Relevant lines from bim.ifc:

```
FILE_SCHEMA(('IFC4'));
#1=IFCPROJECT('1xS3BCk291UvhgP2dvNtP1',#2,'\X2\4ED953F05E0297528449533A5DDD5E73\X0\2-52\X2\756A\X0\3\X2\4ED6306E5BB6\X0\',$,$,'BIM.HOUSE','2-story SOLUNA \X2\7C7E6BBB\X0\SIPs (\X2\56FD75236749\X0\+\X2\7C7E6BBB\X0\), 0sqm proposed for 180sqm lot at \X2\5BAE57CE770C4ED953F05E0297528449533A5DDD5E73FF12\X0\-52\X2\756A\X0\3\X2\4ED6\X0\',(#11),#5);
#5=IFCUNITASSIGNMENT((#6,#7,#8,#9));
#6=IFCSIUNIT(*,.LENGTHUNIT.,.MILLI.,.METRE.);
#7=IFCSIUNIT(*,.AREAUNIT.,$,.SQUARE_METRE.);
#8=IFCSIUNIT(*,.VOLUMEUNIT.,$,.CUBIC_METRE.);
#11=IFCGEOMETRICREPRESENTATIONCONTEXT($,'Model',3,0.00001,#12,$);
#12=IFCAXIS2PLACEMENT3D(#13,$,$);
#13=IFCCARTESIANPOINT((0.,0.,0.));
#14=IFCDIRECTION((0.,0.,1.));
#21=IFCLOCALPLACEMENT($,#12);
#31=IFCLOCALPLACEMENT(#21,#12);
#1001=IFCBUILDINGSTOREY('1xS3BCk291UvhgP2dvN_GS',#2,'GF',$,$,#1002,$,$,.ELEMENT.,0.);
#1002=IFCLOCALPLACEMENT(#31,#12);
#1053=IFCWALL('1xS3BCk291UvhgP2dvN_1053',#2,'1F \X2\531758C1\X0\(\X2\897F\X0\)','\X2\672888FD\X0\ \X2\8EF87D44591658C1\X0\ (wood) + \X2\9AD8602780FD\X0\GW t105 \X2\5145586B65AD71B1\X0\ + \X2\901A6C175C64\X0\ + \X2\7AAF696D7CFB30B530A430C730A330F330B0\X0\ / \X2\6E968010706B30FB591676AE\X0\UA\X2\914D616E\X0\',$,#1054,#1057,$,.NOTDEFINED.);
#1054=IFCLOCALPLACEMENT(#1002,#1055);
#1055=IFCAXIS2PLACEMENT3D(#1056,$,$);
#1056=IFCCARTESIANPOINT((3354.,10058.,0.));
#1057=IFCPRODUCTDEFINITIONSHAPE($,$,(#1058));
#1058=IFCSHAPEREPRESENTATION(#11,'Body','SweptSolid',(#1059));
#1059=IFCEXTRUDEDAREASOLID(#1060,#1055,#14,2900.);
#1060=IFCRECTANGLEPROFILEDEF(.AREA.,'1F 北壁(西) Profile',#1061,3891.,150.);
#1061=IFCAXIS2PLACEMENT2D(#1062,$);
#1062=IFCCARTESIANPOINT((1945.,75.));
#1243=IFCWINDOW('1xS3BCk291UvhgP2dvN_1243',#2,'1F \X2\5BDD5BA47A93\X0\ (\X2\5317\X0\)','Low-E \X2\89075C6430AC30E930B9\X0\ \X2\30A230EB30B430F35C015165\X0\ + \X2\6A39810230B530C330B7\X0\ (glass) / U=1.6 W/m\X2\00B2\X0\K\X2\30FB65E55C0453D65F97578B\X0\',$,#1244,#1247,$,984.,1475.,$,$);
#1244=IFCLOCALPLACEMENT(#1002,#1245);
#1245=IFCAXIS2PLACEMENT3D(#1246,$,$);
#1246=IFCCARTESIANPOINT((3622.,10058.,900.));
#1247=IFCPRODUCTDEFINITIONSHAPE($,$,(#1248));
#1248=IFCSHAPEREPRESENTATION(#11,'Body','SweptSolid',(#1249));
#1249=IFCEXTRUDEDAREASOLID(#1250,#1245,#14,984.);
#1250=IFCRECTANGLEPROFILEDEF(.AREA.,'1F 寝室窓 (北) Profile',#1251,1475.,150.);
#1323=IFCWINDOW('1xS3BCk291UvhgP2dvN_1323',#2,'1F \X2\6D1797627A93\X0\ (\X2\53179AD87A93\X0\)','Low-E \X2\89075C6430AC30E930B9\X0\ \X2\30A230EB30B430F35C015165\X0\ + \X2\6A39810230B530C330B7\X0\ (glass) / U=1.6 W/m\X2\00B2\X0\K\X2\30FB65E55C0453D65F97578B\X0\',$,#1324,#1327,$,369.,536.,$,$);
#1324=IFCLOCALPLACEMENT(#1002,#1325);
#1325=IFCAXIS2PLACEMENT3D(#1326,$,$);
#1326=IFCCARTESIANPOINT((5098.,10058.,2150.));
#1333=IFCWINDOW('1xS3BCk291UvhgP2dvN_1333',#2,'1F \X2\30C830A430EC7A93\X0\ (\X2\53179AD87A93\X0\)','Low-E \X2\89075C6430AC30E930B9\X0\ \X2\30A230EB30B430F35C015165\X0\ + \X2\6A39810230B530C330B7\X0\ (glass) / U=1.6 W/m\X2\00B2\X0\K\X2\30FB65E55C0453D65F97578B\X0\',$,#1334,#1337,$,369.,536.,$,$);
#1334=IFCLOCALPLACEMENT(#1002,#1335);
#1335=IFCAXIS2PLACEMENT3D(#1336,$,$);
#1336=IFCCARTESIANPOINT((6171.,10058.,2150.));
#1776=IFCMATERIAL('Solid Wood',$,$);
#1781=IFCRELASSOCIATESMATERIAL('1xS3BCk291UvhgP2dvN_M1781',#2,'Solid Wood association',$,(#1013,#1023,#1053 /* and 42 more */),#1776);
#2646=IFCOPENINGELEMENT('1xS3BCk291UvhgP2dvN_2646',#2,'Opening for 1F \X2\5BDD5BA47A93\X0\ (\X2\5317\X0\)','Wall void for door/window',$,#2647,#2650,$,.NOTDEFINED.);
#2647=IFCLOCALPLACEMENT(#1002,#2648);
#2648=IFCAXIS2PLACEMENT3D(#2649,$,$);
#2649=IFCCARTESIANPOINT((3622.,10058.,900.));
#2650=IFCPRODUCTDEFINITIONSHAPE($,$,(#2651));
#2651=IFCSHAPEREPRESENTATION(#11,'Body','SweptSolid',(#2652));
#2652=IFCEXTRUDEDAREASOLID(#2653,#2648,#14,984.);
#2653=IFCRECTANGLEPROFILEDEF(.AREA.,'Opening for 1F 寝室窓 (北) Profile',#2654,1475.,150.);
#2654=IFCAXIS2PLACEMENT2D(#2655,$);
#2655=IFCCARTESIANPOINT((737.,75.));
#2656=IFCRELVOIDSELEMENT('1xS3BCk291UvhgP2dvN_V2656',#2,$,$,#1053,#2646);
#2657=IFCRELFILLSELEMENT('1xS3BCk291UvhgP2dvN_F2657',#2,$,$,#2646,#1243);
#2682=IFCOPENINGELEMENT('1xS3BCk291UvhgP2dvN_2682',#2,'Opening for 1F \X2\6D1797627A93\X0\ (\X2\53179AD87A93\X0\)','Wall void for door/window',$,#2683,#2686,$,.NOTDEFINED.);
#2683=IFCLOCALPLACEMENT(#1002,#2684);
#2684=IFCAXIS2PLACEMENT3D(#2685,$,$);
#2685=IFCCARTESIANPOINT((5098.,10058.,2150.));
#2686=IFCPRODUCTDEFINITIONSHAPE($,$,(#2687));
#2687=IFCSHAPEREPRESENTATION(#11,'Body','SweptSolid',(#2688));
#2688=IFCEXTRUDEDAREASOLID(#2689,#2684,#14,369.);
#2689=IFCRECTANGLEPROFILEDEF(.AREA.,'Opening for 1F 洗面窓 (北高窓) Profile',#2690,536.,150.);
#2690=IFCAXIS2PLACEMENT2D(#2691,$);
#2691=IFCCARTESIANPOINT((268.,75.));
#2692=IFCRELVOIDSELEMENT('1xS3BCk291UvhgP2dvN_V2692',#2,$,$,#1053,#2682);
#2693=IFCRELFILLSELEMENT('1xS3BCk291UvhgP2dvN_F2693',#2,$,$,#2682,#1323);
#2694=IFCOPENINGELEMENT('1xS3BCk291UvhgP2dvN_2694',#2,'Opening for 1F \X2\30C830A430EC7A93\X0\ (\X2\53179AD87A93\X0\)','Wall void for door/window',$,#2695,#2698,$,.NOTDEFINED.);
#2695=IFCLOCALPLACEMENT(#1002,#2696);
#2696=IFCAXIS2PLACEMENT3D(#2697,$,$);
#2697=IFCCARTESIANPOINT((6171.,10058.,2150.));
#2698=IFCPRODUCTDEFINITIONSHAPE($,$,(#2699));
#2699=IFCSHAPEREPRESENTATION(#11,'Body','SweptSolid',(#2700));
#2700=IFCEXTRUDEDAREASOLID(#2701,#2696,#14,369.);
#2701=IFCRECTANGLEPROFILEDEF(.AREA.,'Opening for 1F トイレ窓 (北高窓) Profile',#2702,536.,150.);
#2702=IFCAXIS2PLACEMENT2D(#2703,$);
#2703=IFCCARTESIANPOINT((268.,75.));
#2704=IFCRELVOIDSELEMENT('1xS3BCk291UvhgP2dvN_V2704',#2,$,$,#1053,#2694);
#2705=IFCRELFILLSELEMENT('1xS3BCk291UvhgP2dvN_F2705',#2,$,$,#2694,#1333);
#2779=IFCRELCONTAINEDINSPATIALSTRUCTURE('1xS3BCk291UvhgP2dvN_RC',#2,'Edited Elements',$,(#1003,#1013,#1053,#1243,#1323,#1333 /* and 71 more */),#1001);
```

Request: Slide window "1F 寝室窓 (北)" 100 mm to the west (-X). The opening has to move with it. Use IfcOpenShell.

```python
import ifcopenshell
import ifcopenshell.api.geometry
import ifcopenshell.util.placement

model = ifcopenshell.open("bim.ifc")

window = model.by_guid("1xS3BCk291UvhgP2dvN_1243")
opening = window.FillsVoids[0].RelatingOpeningElement
wall = opening.VoidsElements[0].RelatingBuildingElement

wall_matrix = ifcopenshell.util.placement.get_local_placement(wall.ObjectPlacement)
shift = wall_matrix[:3, 0] * -100.0
before = ifcopenshell.util.placement.get_local_placement(window.ObjectPlacement)[:3, 3].copy()

# The window is not placed relative to its opening, so move both.
for product in (opening, window):
    matrix = ifcopenshell.util.placement.get_local_placement(product.ObjectPlacement)
    matrix[:3, 3] += shift
    ifcopenshell.api.geometry.edit_object_placement(model, product=product, matrix=matrix, is_si=False)

after = ifcopenshell.util.placement.get_local_placement(window.ObjectPlacement)[:3, 3]
print("window moved by", (after - before).round(3) + 0.0)

model.write("bim_rev.ifc")
```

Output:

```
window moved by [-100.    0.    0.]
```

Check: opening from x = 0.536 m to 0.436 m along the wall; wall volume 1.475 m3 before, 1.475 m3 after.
